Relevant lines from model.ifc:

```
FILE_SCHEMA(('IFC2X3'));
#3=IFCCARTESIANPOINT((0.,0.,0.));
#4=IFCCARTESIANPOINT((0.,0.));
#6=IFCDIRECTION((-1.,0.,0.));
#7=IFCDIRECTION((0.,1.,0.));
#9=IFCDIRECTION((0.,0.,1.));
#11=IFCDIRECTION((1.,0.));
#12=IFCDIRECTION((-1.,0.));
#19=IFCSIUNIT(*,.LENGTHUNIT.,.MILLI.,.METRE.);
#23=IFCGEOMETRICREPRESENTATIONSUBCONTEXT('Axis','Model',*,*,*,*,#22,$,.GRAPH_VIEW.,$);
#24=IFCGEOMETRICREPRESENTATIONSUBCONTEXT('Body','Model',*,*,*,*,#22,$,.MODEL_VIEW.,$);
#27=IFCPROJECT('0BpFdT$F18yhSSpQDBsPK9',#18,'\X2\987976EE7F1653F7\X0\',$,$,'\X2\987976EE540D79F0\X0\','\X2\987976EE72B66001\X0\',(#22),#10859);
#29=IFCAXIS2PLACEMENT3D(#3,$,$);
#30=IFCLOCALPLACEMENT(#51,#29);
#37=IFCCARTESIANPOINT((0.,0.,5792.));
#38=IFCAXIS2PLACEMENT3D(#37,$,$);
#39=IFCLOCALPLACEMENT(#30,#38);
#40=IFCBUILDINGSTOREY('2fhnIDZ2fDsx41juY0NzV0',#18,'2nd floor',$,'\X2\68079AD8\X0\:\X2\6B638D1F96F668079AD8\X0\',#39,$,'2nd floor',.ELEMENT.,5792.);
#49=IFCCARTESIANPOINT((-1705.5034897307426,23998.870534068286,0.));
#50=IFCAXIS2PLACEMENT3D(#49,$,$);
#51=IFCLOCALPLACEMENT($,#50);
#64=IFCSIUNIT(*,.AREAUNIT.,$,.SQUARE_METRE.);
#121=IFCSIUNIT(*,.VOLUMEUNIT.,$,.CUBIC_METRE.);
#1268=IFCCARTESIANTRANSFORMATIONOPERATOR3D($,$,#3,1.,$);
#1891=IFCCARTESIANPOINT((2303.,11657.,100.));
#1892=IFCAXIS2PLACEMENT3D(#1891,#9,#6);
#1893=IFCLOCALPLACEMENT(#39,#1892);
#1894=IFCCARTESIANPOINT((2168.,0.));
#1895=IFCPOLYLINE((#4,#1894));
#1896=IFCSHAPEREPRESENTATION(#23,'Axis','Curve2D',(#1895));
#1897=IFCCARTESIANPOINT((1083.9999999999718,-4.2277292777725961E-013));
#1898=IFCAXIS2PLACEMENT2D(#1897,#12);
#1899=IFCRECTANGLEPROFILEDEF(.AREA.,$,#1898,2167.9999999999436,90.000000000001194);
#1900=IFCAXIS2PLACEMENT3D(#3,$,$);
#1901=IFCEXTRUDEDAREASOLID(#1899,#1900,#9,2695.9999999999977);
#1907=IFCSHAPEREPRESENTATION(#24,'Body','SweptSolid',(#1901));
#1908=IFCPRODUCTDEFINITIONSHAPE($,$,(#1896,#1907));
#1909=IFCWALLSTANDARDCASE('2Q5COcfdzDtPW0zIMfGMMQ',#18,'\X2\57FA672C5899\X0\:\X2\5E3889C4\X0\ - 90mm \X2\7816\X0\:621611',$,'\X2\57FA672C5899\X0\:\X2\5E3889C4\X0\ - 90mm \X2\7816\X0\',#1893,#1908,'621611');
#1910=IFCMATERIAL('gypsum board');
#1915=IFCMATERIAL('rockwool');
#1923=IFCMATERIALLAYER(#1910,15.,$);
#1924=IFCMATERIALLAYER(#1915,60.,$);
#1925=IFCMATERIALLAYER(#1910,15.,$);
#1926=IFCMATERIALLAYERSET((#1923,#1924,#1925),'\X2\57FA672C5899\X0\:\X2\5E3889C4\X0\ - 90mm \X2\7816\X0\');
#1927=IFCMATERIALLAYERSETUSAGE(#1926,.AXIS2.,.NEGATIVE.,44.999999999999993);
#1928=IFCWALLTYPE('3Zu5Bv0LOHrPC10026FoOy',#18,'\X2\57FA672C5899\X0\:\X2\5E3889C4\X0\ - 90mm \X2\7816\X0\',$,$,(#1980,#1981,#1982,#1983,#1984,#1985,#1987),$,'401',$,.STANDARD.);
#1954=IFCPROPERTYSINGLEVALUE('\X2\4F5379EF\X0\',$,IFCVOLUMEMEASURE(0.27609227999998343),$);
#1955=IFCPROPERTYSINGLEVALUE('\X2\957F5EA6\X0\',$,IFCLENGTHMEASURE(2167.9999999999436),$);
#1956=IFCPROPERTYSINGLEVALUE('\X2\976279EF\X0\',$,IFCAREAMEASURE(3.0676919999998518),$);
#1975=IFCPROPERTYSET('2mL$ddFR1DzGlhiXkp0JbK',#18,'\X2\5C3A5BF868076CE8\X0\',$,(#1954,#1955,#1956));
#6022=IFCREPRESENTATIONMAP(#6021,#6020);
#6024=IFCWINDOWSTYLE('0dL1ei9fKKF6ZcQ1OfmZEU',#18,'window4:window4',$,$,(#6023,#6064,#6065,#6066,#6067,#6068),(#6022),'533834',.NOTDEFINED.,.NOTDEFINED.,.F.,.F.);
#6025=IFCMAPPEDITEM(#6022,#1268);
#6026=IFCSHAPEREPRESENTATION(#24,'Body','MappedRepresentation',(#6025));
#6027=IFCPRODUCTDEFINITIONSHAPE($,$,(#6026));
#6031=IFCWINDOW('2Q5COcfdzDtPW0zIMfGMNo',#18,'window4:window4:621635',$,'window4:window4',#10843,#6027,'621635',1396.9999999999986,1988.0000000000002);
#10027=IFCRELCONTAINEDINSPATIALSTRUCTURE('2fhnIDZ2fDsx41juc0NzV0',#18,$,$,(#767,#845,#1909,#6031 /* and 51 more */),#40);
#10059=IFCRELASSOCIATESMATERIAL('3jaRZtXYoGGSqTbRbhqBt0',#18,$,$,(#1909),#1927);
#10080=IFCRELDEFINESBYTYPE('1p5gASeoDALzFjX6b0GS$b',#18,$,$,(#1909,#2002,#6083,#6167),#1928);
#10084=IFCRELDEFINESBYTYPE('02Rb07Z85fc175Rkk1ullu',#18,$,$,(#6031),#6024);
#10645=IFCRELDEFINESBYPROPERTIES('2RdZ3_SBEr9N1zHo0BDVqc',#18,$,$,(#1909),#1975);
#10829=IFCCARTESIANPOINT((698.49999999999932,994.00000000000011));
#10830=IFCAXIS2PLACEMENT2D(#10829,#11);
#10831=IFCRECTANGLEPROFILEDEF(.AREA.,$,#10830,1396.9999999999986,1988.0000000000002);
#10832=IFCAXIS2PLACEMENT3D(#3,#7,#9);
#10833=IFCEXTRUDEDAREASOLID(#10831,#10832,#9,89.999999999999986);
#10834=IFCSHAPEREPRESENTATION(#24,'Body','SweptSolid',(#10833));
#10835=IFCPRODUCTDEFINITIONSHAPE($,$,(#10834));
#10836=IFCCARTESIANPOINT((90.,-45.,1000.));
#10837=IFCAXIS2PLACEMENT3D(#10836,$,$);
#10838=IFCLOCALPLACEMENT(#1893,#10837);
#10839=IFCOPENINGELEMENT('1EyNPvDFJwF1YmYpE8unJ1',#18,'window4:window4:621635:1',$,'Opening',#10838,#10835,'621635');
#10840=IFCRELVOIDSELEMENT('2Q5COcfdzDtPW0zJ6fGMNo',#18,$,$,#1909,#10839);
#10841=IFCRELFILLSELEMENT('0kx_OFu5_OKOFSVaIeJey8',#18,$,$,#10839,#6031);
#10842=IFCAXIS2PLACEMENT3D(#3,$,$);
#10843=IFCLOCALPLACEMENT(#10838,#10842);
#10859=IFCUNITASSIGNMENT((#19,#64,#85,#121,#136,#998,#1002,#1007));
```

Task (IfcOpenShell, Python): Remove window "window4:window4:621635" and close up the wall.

```python
import ifcopenshell
import ifcopenshell.api.feature
import ifcopenshell.api.pset
import ifcopenshell.api.root
import ifcopenshell.geom
import ifcopenshell.util.element
import ifcopenshell.util.shape
import ifcopenshell.util.unit

model = ifcopenshell.open("model.ifc")
area_scale = ifcopenshell.util.unit.calculate_unit_scale(model, "AREAUNIT")
volume_scale = ifcopenshell.util.unit.calculate_unit_scale(model, "VOLUMEUNIT")
settings = ifcopenshell.geom.settings()


def volume(element):
    """Net volume in cubic metres, openings subtracted."""
    shape = ifcopenshell.geom.create_shape(settings, element)
    return ifcopenshell.util.shape.get_volume(shape.geometry)


window = model.by_id(6031)
opening = window.FillsVoids[0].RelatingOpeningElement
wall = opening.VoidsElements[0].RelatingBuildingElement
before = volume(wall)

ifcopenshell.api.root.remove_product(model, product=window)
ifcopenshell.api.feature.remove_feature(model, feature=opening)

after = volume(wall)
thickness = 0.09  # wall thickness in metres

# Update the wall's stored quantities.
pset = model.by_id(ifcopenshell.util.element.get_pset(wall, "尺寸标注", should_inherit=False)["id"])
ifcopenshell.api.pset.edit_pset(model, pset=pset, properties={
    "体积": model.create_entity("IfcVolumeMeasure", after / volume_scale),
    "面积": model.create_entity("IfcAreaMeasure", after / thickness / area_scale),
})

print(f"wall volume {before:.3f} -> {after:.3f} m3")

model.write("model-out.ifc")
```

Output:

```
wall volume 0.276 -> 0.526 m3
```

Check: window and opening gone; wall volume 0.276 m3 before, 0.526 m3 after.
